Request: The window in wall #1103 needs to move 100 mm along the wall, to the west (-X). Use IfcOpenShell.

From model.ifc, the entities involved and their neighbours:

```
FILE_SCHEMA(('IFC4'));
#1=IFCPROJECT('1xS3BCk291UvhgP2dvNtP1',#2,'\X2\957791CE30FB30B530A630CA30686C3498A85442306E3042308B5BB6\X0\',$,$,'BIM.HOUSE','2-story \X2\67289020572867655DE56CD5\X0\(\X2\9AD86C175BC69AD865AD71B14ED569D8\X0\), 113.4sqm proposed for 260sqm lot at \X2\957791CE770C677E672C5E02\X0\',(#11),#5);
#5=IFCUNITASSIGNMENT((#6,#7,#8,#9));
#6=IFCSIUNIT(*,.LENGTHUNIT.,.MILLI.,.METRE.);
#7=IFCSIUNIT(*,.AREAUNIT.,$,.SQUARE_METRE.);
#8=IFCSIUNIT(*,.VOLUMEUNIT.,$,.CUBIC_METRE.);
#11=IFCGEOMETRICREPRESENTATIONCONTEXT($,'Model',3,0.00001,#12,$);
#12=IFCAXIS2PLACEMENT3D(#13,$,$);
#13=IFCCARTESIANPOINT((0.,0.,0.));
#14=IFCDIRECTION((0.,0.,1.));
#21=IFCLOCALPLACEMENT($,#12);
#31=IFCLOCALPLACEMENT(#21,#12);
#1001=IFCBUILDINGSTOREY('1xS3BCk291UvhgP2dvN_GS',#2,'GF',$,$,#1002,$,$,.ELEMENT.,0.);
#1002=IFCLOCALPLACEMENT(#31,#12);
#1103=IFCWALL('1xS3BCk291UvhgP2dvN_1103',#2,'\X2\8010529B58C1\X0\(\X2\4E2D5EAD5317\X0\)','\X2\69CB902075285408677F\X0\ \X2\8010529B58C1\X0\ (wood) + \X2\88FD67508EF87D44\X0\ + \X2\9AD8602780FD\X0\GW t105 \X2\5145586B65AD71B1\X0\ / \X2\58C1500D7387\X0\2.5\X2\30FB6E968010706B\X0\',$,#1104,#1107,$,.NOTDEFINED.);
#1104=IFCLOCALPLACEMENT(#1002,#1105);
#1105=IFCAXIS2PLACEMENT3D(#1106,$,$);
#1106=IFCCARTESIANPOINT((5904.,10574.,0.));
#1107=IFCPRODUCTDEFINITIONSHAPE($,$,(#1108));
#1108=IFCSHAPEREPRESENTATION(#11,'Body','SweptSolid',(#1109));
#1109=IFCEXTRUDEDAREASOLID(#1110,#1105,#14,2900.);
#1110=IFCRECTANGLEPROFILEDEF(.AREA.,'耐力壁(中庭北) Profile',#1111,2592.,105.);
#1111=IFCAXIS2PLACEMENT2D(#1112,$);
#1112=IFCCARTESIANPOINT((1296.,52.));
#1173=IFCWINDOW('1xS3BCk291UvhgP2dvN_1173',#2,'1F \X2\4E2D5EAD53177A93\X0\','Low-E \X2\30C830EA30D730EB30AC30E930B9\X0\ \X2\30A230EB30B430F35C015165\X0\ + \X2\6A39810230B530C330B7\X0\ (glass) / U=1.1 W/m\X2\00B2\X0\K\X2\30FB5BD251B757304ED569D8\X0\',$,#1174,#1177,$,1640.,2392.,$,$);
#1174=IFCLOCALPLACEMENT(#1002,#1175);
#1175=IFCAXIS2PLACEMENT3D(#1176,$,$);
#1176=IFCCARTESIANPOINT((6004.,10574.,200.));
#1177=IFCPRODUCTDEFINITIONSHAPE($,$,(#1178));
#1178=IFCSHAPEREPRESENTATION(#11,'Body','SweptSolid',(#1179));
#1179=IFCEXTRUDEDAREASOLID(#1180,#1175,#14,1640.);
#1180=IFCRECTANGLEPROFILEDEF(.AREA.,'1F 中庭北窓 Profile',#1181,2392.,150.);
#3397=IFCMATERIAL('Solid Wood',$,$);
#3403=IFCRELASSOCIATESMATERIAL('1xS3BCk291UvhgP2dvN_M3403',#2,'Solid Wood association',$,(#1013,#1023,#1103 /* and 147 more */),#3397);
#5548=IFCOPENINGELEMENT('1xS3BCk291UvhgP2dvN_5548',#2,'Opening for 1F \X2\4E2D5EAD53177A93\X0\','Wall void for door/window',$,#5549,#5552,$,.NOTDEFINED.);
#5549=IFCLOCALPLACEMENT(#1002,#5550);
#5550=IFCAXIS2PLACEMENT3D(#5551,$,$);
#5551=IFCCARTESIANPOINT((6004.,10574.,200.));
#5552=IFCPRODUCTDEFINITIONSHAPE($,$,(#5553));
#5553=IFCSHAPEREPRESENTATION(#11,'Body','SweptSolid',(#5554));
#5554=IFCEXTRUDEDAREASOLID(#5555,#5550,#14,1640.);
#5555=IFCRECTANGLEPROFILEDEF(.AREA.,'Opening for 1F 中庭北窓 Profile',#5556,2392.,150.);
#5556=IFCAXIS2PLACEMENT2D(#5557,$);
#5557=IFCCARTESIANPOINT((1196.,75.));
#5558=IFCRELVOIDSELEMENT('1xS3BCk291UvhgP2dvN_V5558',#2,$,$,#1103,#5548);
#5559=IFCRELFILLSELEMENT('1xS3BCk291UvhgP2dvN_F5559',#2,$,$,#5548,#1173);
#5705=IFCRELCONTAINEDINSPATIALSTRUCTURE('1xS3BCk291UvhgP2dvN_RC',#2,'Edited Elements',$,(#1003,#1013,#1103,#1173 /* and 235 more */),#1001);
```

```python
import ifcopenshell
import ifcopenshell.api.geometry
import ifcopenshell.util.placement

model = ifcopenshell.open("model.ifc")

window = model.by_guid("1xS3BCk291UvhgP2dvN_1173")
opening = window.FillsVoids[0].RelatingOpeningElement
wall = opening.VoidsElements[0].RelatingBuildingElement

wall_matrix = ifcopenshell.util.placement.get_local_placement(wall.ObjectPlacement)
shift = wall_matrix[:3, 0] * -100.0
before = ifcopenshell.util.placement.get_local_placement(window.ObjectPlacement)[:3, 3].copy()

# The window is not placed relative to its opening, so move both.
for product in (opening, window):
    matrix = ifcopenshell.util.placement.get_local_placement(product.ObjectPlacement)
    matrix[:3, 3] += shift
    ifcopenshell.api.geometry.edit_object_placement(model, product=product, matrix=matrix, is_si=False)

after = ifcopenshell.util.placement.get_local_placement(window.ObjectPlacement)[:3, 3]
print("window moved by", (after - before).round(3) + 0.0)

model.write("model-out.ifc")
```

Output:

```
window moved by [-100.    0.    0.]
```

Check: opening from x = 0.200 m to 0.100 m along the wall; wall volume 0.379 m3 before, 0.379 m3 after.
